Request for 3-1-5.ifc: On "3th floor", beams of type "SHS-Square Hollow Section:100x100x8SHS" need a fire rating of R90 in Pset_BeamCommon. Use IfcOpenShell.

First a look at what the model holds.

```python
import ifcopenshell
import ifcopenshell.util.element

model = ifcopenshell.open("3-1-5.ifc")
print(model.schema)
storey = next(s for s in model.by_type("IfcBuildingStorey") if s.Name == "3th floor")
beams = [e for e in ifcopenshell.util.element.get_decomposition(storey) if e.is_a("IfcBeam")]
seen = {}
for e in beams:
    element_type = ifcopenshell.util.element.get_type(e)
    key = (element_type.Name if element_type != e and element_type else None, ifcopenshell.util.element.get_pset(e, "Pset_BeamCommon", "FireRating"))
    seen[key] = seen.get(key, 0) + 1
for (name, value), count in sorted(seen.items(), key=str):
    print(count, "x", name, "|", value)
```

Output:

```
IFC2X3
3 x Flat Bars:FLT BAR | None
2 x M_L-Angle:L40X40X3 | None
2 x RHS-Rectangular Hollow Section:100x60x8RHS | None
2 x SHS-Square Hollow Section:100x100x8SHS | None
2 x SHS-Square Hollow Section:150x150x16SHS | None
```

```python
import ifcopenshell
import ifcopenshell.api.pset
import ifcopenshell.util.element

model = ifcopenshell.open("3-1-5.ifc")

storey = next(s for s in model.by_type("IfcBuildingStorey") if s.Name == "3th floor")
beams = [e for e in ifcopenshell.util.element.get_decomposition(storey) if e.is_a("IfcBeam")]

count = 0
for e in beams:
    element_type = ifcopenshell.util.element.get_type(e)
    if element_type in (None, e) or element_type.Name != "SHS-Square Hollow Section:100x100x8SHS":
        continue
    # add_pset returns the element's existing set when there is one.
    pset = ifcopenshell.api.pset.add_pset(model, product=e, name="Pset_BeamCommon")
    ifcopenshell.api.pset.edit_pset(model, pset=pset, properties={"FireRating": "R90"})
    count += 1

print(count, "beams updated")

model.write("3-1-5_updated.ifc")
```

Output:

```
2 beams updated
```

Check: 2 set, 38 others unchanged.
